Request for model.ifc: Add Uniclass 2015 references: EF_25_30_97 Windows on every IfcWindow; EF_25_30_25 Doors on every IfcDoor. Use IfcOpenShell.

First a look at what the model holds.

```python
import ifcopenshell

model = ifcopenshell.open("model.ifc")
print(model.schema)
print("classifications:", [c.Name for c in model.by_type("IfcClassification")])
for ifc_class in ("IfcDoor", "IfcRoof", "IfcStair", "IfcWall", "IfcWindow"):
    print(ifc_class, len(model.by_type(ifc_class)))
```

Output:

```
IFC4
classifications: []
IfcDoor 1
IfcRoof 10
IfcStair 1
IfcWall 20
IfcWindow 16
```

```python
import ifcopenshell
import ifcopenshell.api.classification

model = ifcopenshell.open("model.ifc")

system = ifcopenshell.api.classification.add_classification(model, classification="Uniclass 2015")

codes = {
    "IfcWindow": ("EF_25_30_97", "Windows"),
    "IfcDoor": ("EF_25_30_25", "Doors"),
}
for ifc_class, (code, name) in codes.items():
    products = model.by_type(ifc_class)
    ifcopenshell.api.classification.add_reference(
        model, products=products, classification=system, identification=code, name=name
    )
    print(code, len(products))

model.write("model_edited.ifc")
```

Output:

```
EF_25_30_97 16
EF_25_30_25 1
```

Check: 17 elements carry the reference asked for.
